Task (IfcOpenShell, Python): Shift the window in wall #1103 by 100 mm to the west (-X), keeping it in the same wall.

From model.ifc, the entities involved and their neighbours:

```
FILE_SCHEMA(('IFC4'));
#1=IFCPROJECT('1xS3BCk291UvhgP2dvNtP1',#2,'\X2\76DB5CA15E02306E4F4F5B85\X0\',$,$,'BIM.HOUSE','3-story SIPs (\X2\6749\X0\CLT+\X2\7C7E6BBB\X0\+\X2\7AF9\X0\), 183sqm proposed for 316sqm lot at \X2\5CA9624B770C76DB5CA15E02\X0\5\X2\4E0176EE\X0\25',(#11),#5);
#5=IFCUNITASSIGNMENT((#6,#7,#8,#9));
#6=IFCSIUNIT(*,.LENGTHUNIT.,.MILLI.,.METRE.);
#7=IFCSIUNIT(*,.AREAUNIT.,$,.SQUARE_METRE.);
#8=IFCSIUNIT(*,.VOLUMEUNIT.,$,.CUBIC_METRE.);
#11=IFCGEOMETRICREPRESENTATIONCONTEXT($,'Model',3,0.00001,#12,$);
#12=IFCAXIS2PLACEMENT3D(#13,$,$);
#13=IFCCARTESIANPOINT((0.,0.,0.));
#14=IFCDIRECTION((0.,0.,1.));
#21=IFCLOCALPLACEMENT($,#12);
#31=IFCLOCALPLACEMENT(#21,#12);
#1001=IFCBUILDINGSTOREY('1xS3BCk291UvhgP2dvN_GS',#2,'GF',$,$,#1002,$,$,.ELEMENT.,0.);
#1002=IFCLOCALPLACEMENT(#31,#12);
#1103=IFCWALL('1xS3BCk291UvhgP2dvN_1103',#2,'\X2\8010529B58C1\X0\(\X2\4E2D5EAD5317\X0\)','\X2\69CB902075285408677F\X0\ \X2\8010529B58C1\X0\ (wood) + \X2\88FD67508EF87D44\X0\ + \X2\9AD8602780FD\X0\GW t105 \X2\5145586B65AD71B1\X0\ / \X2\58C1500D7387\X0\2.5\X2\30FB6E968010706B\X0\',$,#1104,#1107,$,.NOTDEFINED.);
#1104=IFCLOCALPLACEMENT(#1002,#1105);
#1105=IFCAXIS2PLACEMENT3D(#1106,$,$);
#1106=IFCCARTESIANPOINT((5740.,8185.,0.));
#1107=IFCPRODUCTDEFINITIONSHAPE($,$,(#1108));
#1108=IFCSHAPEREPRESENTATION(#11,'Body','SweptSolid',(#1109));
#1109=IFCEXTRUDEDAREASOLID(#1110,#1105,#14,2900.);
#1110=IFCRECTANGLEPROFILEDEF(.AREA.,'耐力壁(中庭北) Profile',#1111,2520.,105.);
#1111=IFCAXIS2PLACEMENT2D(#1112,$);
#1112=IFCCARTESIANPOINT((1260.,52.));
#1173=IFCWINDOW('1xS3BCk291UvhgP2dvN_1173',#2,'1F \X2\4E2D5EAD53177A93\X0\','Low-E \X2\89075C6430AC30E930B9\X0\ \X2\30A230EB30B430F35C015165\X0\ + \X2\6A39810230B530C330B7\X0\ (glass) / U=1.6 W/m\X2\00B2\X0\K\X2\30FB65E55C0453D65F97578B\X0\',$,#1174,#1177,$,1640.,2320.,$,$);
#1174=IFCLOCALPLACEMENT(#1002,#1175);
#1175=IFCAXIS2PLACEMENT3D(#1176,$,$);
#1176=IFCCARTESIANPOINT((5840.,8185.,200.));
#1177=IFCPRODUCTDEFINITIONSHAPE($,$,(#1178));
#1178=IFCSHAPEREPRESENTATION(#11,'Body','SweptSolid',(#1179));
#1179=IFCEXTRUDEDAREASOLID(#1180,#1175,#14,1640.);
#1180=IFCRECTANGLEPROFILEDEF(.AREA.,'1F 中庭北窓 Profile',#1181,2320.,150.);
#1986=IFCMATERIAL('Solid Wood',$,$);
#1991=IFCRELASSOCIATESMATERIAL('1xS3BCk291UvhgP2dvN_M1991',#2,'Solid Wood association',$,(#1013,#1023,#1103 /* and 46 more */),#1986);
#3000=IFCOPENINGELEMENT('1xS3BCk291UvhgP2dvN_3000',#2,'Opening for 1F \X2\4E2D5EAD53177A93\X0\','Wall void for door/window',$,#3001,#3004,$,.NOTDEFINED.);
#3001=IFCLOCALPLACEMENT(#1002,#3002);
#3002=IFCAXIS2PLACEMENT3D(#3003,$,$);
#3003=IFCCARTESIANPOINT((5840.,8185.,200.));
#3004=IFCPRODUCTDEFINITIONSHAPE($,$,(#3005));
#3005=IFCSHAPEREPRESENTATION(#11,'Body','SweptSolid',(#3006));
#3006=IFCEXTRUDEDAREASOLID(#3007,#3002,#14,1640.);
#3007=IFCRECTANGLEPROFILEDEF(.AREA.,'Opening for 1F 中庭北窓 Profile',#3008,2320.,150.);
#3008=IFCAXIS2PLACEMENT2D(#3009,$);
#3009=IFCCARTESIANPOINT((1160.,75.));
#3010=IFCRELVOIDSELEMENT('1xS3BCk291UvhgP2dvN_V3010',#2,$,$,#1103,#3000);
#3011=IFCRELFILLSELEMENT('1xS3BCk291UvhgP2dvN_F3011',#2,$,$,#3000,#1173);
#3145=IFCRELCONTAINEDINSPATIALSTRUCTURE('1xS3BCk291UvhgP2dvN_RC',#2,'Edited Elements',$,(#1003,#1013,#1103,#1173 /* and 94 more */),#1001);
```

```python
import ifcopenshell
import ifcopenshell.api.geometry
import ifcopenshell.util.placement
import ifcopenshell.util.unit

model = ifcopenshell.open("model.ifc")
unit_scale = ifcopenshell.util.unit.calculate_unit_scale(model)

window = model.by_guid("1xS3BCk291UvhgP2dvN_1173")
opening = window.FillsVoids[0].RelatingOpeningElement
wall = opening.VoidsElements[0].RelatingBuildingElement

wall_matrix = ifcopenshell.util.placement.get_local_placement(wall.ObjectPlacement)
shift = wall_matrix[:3, 0] * -0.1 / unit_scale
before = ifcopenshell.util.placement.get_local_placement(window.ObjectPlacement)[:3, 3].copy()

# The window is not placed relative to its opening, so move both.
for product in (opening, window):
    matrix = ifcopenshell.util.placement.get_local_placement(product.ObjectPlacement)
    matrix[:3, 3] += shift
    ifcopenshell.api.geometry.edit_object_placement(model, product=product, matrix=matrix, is_si=False)

after = ifcopenshell.util.placement.get_local_placement(window.ObjectPlacement)[:3, 3]
print("window moved by", (after - before).round(3) + 0.0)

model.write("model-out.ifc")
```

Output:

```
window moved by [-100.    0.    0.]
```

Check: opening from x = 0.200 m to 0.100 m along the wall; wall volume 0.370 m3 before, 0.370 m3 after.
